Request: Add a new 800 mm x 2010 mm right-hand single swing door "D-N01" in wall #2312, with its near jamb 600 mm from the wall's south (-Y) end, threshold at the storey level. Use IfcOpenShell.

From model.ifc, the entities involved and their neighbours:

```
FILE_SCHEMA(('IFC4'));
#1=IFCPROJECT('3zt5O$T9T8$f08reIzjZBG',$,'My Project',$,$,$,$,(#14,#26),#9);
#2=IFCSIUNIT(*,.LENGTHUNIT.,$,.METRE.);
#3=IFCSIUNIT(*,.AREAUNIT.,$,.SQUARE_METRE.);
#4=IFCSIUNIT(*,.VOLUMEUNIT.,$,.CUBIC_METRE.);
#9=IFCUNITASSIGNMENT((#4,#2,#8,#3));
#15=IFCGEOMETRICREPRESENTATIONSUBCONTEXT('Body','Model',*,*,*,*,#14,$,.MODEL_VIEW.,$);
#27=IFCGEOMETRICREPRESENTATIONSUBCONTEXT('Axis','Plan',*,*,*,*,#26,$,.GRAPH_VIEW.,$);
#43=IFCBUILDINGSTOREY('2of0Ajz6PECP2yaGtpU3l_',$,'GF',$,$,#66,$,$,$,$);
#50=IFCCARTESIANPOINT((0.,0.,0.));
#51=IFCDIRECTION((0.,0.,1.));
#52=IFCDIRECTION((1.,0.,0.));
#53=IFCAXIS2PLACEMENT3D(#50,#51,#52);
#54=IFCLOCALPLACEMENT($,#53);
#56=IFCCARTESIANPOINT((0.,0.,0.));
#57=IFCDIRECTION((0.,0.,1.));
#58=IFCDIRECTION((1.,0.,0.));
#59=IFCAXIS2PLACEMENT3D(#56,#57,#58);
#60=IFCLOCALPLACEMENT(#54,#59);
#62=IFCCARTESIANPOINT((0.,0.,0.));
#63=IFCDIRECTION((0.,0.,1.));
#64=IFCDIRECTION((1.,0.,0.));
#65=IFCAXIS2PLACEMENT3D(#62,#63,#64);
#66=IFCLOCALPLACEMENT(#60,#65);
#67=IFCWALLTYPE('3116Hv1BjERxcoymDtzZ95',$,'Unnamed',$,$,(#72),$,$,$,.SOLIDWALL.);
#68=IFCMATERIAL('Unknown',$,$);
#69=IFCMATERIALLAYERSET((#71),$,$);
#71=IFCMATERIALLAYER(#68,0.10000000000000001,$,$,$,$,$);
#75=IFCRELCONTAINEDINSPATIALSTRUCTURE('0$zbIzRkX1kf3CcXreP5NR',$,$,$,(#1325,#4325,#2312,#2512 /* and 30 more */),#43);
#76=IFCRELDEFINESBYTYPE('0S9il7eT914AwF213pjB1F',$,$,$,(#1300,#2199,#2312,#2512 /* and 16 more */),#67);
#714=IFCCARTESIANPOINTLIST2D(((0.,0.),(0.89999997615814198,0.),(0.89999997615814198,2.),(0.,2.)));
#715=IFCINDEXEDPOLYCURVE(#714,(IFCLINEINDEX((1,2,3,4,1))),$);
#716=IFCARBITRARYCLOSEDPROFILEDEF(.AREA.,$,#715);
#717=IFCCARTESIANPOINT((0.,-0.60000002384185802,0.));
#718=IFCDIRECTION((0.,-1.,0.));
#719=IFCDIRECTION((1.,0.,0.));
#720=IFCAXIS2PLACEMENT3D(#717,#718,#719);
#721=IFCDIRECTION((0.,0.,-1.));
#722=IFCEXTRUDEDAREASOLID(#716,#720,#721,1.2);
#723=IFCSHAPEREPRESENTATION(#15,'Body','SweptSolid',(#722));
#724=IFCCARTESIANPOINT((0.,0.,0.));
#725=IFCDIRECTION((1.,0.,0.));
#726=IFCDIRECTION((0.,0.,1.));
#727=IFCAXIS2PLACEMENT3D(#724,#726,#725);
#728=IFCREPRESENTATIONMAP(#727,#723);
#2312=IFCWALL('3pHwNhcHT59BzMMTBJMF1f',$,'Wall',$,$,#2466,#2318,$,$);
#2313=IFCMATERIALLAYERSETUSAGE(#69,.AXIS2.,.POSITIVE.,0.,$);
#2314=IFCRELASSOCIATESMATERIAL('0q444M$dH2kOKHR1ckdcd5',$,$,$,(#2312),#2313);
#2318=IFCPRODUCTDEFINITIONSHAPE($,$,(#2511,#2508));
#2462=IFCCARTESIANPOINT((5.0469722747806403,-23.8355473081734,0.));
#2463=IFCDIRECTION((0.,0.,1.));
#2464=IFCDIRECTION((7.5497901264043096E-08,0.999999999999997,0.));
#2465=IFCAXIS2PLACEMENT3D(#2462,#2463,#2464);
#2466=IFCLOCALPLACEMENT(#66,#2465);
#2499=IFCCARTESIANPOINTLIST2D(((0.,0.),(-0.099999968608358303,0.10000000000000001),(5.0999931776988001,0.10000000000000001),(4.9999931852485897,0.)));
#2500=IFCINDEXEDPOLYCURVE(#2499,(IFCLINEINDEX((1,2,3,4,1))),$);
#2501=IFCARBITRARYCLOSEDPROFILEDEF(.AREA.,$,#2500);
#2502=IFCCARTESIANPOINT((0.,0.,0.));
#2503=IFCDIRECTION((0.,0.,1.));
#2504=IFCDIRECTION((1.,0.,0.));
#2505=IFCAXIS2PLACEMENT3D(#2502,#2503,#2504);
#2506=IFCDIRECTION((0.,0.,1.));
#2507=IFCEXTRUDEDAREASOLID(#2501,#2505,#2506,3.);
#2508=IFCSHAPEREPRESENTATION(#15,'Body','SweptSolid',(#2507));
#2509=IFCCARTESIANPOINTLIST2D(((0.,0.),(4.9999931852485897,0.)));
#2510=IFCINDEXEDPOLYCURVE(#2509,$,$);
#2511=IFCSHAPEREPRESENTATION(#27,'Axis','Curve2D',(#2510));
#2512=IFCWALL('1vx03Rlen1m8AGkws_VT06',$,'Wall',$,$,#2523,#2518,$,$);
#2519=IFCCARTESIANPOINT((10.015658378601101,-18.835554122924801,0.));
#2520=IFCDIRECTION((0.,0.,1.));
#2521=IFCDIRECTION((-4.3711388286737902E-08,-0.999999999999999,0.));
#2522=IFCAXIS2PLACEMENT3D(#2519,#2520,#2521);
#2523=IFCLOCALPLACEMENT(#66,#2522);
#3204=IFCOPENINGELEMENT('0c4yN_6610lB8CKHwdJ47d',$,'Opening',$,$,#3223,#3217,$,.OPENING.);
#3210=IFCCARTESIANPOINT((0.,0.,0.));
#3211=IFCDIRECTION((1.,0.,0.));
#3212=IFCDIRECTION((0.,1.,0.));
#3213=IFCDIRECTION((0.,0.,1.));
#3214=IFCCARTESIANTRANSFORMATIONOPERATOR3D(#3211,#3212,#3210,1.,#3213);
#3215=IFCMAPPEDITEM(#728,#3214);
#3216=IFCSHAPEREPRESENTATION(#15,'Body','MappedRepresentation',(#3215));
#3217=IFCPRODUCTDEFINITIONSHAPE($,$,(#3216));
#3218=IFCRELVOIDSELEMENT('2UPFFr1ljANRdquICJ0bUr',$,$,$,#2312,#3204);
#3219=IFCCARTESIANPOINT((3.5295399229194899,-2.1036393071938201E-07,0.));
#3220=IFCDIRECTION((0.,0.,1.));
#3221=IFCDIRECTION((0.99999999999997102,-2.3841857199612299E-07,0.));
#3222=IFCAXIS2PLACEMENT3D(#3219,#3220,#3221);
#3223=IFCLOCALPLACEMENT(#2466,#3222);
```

```python
import numpy as np
import ifcopenshell
import ifcopenshell.api.feature
import ifcopenshell.api.geometry
import ifcopenshell.api.root
import ifcopenshell.api.spatial
import ifcopenshell.geom
import ifcopenshell.util.element
import ifcopenshell.util.placement
import ifcopenshell.util.representation
import ifcopenshell.util.shape
import ifcopenshell.util.unit

model = ifcopenshell.open("model.ifc")
unit_scale = ifcopenshell.util.unit.calculate_unit_scale(model)
settings = ifcopenshell.geom.settings()


def volume(element):
    """Net volume in cubic metres, openings subtracted."""
    shape = ifcopenshell.geom.create_shape(settings, element)
    return ifcopenshell.util.shape.get_volume(shape.geometry)


wall = model.by_guid("3pHwNhcHT59BzMMTBJMF1f")
storey = ifcopenshell.util.element.get_container(wall, ifc_class="IfcBuildingStorey")
context = ifcopenshell.util.representation.get_context(model, "Model", "Body", "MODEL_VIEW")
before = volume(wall)

width, height, from_end, sill = 0.8, 2.01, 0.6, 0.0  # metres

# The wall runs along its own X axis, and the end named is its -X end.
wall_shape = ifcopenshell.geom.create_shape(settings, wall)
x, y, z = ifcopenshell.util.shape.get_vertices(wall_shape.geometry).T
start = x.min() + from_end
face, thickness = float(y.min()), float(y.max() - y.min())
wall_matrix = ifcopenshell.util.placement.get_local_placement(wall.ObjectPlacement)
level = ifcopenshell.util.placement.get_local_placement(storey.ObjectPlacement)[2, 3]


def in_wall(x, y):
    """Placement at x, y metres in the wall's axes, at sill height."""
    matrix = wall_matrix.copy()
    matrix[:, 3] = wall_matrix @ np.array([x / unit_scale, y / unit_scale, 0.0, 1.0])
    matrix[2, 3] = level + sill / unit_scale
    return matrix


# Opening: a box that overshoots both wall faces by 50 mm.
opening = ifcopenshell.api.root.create_entity(model, ifc_class="IfcOpeningElement", predefined_type="OPENING")
box = ifcopenshell.api.geometry.add_wall_representation(
    model, context=context, length=width, height=height, thickness=thickness + 0.1
)
ifcopenshell.api.geometry.assign_representation(model, product=opening, representation=box)
ifcopenshell.api.geometry.edit_object_placement(model, product=opening, matrix=in_wall(start, face - 0.05), is_si=False)
ifcopenshell.api.feature.add_feature(model, feature=opening, element=wall)

door = ifcopenshell.api.root.create_entity(model, ifc_class="IfcDoor", name="D-N01", predefined_type="DOOR")
door.OverallWidth, door.OverallHeight = width / unit_scale, height / unit_scale
door.OperationType = "SINGLE_SWING_RIGHT"
body = ifcopenshell.api.geometry.add_door_representation(
    model,
    context=context,
    overall_width=door.OverallWidth,
    overall_height=door.OverallHeight,
    operation_type="SINGLE_SWING_RIGHT",
    lining_properties={"LiningDepth": thickness / unit_scale, "ThresholdDepth": thickness / unit_scale},
)
ifcopenshell.api.geometry.assign_representation(model, product=door, representation=body)
ifcopenshell.api.spatial.assign_container(model, products=[door], relating_structure=storey)
ifcopenshell.api.feature.add_filling(model, opening=opening, element=door)

# The lining spans the wall, so the door starts at the wall face.
ifcopenshell.api.geometry.edit_object_placement(model, product=door, matrix=in_wall(start, face), is_si=False)

after = volume(wall)

print(f"wall volume {before:.3f} -> {after:.3f} m3")

model.write("model_rev.ifc")
```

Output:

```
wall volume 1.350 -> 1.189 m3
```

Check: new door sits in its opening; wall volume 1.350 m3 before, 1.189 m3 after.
